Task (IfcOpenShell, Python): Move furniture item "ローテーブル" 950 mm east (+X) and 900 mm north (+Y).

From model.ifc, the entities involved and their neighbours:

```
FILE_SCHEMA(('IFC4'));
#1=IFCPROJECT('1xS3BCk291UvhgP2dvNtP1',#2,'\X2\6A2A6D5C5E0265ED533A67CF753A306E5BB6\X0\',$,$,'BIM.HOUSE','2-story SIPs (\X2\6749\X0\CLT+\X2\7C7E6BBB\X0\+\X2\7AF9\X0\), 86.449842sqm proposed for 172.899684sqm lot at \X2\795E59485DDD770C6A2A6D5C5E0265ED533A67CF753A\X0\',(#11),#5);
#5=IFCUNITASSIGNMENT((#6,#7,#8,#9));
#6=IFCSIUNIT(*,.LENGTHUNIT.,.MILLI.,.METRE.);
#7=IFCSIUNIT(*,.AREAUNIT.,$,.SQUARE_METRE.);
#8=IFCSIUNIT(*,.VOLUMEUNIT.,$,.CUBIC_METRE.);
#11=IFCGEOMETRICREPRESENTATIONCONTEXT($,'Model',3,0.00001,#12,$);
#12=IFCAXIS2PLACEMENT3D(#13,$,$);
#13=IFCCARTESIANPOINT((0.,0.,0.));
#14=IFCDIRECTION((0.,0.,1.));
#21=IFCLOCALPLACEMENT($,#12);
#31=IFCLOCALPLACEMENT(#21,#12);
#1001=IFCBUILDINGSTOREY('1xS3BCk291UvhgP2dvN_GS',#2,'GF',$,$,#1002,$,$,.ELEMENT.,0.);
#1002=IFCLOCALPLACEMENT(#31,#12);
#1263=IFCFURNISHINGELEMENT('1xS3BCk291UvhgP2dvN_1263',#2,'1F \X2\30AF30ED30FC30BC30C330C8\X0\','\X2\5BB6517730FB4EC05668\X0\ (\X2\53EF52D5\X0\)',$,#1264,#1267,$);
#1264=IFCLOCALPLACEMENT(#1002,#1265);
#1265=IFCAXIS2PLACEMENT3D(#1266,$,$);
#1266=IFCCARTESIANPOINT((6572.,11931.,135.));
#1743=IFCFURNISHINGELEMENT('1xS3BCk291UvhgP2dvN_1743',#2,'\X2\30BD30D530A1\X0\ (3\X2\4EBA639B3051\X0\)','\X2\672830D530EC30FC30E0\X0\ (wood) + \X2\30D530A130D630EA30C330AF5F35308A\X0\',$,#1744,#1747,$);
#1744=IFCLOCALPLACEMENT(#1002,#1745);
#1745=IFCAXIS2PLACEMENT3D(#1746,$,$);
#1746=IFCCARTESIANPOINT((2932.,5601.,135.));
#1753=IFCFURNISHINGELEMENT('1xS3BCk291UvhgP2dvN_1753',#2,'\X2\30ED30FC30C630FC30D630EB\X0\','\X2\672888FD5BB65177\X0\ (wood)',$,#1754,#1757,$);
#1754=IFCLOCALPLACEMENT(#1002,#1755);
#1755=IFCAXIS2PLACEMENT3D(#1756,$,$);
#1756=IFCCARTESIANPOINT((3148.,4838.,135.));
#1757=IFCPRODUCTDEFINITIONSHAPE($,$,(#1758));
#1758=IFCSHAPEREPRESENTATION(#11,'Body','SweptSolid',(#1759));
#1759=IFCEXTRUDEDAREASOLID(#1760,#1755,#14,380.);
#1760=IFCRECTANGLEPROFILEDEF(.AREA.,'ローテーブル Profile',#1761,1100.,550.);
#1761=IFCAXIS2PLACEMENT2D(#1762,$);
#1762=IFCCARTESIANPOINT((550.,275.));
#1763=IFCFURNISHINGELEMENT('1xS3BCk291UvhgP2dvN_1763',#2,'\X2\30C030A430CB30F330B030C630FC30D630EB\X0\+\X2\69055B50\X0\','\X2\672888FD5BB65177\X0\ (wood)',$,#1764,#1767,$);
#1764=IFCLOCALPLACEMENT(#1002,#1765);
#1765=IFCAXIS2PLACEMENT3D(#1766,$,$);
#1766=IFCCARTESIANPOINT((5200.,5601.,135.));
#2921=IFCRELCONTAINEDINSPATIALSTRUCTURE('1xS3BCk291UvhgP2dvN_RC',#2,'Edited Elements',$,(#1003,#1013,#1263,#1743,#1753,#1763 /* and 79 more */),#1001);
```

```python
import ifcopenshell
import ifcopenshell.api.geometry
import ifcopenshell.util.placement
import ifcopenshell.util.unit

model = ifcopenshell.open("model.ifc")
unit_scale = ifcopenshell.util.unit.calculate_unit_scale(model)

item = model.by_id(1753)
matrix = ifcopenshell.util.placement.get_local_placement(item.ObjectPlacement)
matrix[0, 3] += 0.95 / unit_scale
matrix[1, 3] += 0.9 / unit_scale
ifcopenshell.api.geometry.edit_object_placement(model, product=item, matrix=matrix, is_si=False)

print(ifcopenshell.util.placement.get_local_placement(item.ObjectPlacement).round(3) + 0.0)

model.write("model_v2.ifc")
```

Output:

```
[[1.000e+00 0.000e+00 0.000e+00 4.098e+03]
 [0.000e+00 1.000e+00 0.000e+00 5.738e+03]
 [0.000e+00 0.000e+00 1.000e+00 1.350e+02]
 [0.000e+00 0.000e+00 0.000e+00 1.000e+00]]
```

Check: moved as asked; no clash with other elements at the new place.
